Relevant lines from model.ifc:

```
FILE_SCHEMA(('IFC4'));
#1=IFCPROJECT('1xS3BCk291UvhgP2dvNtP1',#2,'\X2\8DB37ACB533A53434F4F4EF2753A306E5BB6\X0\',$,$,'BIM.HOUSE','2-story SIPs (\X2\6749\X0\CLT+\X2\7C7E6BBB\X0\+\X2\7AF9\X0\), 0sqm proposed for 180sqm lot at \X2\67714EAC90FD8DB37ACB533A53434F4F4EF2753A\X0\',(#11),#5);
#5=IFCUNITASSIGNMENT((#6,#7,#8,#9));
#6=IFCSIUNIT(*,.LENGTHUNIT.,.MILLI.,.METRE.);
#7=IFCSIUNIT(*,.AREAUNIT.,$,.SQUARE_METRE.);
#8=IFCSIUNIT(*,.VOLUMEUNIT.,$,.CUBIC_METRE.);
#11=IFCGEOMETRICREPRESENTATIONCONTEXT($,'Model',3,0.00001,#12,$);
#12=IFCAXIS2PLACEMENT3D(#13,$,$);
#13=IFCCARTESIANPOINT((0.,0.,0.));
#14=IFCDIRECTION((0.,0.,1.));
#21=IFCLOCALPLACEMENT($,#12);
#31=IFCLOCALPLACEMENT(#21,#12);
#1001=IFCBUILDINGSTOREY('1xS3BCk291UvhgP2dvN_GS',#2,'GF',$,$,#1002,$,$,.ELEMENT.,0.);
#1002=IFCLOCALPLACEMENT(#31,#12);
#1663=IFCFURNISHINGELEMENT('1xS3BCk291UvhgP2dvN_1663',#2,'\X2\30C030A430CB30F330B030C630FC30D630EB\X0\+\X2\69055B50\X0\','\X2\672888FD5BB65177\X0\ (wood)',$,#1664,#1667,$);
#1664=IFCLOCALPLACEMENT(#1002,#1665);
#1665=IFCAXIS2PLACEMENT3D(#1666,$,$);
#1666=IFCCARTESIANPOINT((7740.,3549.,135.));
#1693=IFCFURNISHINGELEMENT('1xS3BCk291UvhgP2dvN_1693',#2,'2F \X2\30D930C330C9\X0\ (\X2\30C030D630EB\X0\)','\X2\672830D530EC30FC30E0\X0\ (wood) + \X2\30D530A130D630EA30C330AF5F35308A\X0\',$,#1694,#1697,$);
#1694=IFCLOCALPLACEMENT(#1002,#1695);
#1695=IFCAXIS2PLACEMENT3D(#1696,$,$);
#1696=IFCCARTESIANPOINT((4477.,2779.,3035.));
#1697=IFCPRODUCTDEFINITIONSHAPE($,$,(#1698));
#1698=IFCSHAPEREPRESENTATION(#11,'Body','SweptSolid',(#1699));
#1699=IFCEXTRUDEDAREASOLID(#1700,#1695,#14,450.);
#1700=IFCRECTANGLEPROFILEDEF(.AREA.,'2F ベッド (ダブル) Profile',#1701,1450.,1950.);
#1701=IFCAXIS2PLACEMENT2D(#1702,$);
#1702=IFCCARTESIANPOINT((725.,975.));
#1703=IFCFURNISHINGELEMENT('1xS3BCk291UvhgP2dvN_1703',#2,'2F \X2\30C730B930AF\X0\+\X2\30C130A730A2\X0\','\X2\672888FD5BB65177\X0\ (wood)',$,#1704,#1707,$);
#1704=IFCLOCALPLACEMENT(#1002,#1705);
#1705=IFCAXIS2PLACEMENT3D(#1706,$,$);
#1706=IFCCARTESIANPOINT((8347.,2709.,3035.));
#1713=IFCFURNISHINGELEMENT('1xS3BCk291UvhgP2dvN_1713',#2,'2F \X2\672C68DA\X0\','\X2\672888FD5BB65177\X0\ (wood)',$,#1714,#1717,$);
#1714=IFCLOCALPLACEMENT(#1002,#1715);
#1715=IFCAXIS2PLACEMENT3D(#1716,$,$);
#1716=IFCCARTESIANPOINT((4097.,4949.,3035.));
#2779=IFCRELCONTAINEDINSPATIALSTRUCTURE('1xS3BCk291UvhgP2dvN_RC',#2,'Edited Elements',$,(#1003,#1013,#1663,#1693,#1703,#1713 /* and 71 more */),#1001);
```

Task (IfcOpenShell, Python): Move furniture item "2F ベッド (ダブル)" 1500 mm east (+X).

```python
import ifcopenshell
import ifcopenshell.api.geometry
import ifcopenshell.util.placement
import ifcopenshell.util.unit

model = ifcopenshell.open("model.ifc")
unit_scale = ifcopenshell.util.unit.calculate_unit_scale(model)

item = model.by_guid("1xS3BCk291UvhgP2dvN_1693")
matrix = ifcopenshell.util.placement.get_local_placement(item.ObjectPlacement)
matrix[0, 3] += 1.5 / unit_scale
ifcopenshell.api.geometry.edit_object_placement(model, product=item, matrix=matrix, is_si=False)

print(ifcopenshell.util.placement.get_local_placement(item.ObjectPlacement).round(3) + 0.0)

model.write("model_v2.ifc")
```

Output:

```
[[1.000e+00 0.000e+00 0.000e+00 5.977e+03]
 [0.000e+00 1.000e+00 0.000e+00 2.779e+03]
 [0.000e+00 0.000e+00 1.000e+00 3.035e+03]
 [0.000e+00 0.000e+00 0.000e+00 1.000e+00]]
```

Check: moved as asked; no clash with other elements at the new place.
